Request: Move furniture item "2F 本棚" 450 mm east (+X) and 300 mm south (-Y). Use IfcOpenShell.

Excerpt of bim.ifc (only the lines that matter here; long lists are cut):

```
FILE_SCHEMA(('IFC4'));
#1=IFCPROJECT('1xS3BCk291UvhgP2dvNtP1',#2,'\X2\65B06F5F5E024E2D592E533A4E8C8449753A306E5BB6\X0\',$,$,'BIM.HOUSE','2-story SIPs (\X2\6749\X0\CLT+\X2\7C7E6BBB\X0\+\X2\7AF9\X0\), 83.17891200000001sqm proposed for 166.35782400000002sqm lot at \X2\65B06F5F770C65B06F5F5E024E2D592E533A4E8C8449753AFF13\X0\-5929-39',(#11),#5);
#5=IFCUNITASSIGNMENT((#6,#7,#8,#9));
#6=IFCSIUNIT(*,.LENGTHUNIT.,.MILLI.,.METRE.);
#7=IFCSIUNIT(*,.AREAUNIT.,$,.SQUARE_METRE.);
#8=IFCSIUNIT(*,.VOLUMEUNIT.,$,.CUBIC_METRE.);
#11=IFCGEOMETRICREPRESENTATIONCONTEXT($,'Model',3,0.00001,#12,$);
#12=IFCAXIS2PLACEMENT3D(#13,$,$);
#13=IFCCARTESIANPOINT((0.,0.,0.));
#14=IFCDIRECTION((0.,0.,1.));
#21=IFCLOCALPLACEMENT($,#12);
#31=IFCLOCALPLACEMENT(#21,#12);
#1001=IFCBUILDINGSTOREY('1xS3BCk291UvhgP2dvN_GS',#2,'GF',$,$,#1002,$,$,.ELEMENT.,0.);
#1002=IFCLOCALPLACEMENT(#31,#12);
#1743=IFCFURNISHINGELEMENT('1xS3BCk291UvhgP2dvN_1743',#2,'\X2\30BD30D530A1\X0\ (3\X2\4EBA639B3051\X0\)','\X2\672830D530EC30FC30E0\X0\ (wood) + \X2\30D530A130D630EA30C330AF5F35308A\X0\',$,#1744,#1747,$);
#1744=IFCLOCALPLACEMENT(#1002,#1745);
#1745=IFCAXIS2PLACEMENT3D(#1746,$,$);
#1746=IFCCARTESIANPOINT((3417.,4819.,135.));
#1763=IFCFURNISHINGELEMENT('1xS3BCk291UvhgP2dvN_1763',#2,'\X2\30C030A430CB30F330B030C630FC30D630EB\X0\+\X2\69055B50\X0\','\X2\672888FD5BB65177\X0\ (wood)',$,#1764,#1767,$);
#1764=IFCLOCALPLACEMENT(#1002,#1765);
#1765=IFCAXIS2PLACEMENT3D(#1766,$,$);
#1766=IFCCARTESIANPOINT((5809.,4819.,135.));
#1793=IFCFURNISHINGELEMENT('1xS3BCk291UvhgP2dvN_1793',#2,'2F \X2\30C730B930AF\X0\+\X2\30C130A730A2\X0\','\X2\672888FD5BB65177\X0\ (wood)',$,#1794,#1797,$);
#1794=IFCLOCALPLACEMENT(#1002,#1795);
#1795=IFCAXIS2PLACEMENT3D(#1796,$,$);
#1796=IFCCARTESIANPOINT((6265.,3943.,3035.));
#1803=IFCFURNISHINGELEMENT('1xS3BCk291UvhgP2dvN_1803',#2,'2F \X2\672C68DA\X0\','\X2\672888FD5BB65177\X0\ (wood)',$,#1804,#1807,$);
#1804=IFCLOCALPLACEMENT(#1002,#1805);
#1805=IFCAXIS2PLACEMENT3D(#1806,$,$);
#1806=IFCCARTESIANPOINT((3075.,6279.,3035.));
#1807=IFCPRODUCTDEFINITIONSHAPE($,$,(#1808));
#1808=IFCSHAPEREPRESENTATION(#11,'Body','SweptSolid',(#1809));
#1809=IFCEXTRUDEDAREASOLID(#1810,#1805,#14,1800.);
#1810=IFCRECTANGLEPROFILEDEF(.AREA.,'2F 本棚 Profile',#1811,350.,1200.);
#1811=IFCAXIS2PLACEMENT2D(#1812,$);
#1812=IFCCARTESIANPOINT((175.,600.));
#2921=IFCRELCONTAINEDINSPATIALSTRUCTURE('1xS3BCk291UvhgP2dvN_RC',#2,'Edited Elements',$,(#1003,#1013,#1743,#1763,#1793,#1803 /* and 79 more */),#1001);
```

```python
import ifcopenshell
import ifcopenshell.api.geometry
import ifcopenshell.util.placement
import ifcopenshell.util.unit

model = ifcopenshell.open("bim.ifc")
unit_scale = ifcopenshell.util.unit.calculate_unit_scale(model)

item = model.by_id(1803)
matrix = ifcopenshell.util.placement.get_local_placement(item.ObjectPlacement)
matrix[0, 3] += 0.45 / unit_scale
matrix[1, 3] -= 0.3 / unit_scale
ifcopenshell.api.geometry.edit_object_placement(model, product=item, matrix=matrix, is_si=False)

print(ifcopenshell.util.placement.get_local_placement(item.ObjectPlacement).round(3) + 0.0)

model.write("bim_v2.ifc")
```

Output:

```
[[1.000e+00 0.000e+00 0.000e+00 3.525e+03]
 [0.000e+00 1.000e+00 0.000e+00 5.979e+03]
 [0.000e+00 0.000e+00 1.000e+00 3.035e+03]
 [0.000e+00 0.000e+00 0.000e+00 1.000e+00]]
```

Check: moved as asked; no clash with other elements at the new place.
